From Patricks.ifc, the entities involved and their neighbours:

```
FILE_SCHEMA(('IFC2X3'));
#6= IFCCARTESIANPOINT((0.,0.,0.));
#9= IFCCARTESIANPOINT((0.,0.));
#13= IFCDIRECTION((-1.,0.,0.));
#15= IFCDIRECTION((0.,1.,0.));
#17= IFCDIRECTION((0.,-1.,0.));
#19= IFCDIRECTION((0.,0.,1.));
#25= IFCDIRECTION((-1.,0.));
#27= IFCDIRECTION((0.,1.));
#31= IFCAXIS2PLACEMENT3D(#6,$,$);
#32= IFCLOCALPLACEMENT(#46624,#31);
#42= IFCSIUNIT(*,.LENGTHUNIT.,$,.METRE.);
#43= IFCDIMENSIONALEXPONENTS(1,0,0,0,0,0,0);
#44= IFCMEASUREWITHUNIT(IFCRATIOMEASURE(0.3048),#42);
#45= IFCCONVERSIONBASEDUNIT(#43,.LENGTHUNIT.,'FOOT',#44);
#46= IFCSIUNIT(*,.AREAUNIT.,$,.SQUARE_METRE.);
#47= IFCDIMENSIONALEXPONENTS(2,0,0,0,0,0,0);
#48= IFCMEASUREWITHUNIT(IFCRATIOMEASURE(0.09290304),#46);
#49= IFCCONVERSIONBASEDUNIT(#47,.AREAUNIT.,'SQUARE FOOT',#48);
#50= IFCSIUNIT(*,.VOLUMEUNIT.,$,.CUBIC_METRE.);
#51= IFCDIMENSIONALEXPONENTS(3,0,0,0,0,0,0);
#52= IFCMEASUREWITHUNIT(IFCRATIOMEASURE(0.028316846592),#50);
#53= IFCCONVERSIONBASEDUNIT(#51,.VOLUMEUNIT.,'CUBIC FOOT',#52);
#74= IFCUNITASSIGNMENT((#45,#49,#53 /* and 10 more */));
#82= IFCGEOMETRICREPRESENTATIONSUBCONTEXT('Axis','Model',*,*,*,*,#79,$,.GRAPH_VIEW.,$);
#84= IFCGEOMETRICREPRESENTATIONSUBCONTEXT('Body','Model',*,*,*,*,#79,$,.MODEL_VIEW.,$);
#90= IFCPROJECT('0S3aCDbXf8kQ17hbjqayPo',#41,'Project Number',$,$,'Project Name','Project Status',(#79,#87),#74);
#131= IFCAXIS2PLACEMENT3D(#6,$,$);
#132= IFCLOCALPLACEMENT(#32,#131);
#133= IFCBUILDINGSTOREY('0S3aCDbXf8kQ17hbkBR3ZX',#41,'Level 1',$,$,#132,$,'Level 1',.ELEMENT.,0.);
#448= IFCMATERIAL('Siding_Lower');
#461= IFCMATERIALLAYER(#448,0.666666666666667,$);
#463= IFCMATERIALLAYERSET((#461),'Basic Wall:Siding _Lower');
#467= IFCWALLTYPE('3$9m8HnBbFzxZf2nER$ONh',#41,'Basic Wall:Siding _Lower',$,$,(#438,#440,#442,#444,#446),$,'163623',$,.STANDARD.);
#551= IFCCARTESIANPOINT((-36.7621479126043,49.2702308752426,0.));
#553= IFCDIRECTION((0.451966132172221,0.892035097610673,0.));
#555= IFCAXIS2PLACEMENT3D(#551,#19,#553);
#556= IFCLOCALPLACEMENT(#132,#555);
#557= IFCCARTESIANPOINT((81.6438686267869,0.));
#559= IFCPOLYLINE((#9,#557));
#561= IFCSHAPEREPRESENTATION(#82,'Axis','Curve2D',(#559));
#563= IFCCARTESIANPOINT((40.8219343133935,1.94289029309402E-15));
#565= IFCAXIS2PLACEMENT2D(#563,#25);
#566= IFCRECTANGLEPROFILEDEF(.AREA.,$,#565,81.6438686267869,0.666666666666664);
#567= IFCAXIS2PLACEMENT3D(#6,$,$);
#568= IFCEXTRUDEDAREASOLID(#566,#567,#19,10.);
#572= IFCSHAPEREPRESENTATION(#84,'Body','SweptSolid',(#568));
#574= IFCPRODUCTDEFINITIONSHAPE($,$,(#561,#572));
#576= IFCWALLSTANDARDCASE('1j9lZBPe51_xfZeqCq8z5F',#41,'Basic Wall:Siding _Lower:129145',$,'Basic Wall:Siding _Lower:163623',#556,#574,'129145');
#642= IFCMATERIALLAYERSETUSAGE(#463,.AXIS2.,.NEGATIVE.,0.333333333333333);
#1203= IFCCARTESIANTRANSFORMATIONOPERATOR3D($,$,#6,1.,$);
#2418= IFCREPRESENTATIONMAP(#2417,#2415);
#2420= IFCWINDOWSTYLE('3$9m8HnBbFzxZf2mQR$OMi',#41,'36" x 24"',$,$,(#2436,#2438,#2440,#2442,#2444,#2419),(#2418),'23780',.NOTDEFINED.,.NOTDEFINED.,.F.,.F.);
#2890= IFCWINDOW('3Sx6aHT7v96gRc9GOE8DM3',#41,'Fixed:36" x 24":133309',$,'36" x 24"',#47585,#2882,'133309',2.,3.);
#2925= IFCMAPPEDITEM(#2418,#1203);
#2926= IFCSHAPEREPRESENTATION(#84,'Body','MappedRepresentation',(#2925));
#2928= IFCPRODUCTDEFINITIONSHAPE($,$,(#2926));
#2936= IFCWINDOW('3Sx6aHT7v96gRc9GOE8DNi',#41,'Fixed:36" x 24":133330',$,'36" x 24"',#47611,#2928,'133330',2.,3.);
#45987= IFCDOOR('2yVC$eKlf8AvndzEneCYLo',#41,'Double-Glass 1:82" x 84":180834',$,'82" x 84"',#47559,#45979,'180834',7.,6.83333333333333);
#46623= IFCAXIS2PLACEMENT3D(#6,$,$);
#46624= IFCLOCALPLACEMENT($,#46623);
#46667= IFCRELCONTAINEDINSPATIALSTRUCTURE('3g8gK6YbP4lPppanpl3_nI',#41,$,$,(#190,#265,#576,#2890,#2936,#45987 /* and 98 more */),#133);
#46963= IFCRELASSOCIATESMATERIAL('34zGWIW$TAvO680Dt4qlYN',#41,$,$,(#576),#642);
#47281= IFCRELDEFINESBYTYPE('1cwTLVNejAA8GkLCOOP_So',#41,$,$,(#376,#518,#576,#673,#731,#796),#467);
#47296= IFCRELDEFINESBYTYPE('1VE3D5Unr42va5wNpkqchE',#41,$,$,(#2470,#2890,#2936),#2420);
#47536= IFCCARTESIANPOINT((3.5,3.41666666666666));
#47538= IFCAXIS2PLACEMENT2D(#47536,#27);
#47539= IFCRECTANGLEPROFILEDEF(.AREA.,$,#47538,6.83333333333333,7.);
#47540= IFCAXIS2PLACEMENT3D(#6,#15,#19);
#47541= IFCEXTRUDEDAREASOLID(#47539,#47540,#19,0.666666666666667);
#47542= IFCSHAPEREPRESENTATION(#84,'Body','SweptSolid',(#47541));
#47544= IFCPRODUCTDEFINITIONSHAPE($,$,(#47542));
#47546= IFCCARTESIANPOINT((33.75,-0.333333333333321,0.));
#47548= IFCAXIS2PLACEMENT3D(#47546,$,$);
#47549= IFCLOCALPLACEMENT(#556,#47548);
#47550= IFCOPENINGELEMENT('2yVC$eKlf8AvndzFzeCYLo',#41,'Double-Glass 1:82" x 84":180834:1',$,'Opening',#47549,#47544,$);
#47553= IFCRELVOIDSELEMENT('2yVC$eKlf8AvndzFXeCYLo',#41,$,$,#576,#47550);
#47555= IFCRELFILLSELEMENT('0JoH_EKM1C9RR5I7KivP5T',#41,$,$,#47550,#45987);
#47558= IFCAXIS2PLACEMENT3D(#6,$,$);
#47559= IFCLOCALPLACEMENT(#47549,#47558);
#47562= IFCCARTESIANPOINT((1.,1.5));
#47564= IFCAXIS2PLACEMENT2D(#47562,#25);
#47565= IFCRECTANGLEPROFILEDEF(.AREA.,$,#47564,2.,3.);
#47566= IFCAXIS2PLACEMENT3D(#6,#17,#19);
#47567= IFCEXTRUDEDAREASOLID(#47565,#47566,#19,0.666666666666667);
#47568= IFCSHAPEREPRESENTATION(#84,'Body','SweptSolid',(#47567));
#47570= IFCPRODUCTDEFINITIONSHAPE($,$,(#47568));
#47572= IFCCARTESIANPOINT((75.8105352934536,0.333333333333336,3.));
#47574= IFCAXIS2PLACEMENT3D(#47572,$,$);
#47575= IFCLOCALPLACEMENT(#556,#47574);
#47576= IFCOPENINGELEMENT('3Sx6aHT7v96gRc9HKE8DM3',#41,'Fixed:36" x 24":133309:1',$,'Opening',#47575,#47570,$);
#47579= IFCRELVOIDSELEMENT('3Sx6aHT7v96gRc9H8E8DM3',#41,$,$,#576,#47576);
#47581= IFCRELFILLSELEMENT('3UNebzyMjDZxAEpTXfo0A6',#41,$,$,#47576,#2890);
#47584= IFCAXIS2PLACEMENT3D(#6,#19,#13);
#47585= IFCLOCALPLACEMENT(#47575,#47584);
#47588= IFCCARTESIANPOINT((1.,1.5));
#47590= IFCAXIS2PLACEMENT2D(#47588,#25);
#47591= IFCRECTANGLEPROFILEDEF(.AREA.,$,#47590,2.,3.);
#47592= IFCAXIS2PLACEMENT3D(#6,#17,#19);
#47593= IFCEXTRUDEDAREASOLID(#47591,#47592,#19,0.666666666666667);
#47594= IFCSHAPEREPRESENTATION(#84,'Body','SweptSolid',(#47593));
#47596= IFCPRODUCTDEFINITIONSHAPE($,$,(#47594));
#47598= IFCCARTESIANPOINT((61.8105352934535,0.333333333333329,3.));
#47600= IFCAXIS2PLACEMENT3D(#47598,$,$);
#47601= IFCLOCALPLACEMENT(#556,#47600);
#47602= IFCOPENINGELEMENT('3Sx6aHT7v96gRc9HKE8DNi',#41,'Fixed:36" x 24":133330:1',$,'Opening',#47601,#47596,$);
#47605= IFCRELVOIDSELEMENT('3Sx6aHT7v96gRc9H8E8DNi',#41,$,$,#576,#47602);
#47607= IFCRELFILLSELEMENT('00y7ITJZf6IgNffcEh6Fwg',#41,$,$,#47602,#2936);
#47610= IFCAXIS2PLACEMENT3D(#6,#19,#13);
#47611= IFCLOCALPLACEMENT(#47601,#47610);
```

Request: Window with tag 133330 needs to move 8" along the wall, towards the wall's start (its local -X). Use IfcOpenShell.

```python
import ifcopenshell
import ifcopenshell.api.geometry
import ifcopenshell.util.placement
import ifcopenshell.util.unit

model = ifcopenshell.open("Patricks.ifc")
unit_scale = ifcopenshell.util.unit.calculate_unit_scale(model)

window = model.by_guid("3Sx6aHT7v96gRc9GOE8DNi")
opening = window.FillsVoids[0].RelatingOpeningElement
wall = opening.VoidsElements[0].RelatingBuildingElement

wall_matrix = ifcopenshell.util.placement.get_local_placement(wall.ObjectPlacement)
shift = wall_matrix[:3, 0] * -8 * 0.0254 / unit_scale
before = ifcopenshell.util.placement.get_local_placement(window.ObjectPlacement)[:3, 3].copy()

# The window is placed relative to its opening, so it follows when the opening moves.
matrix = ifcopenshell.util.placement.get_local_placement(opening.ObjectPlacement)
matrix[:3, 3] += shift
ifcopenshell.api.geometry.edit_object_placement(
    model, product=opening, matrix=matrix, is_si=False, should_transform_children=True
)

after = ifcopenshell.util.placement.get_local_placement(window.ObjectPlacement)[:3, 3]
print("window moved by", (after - before).round(3) + 0.0)

model.write("Patricks-out.ifc")
```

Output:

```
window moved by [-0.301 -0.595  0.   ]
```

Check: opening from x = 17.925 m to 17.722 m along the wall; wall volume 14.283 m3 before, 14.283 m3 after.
